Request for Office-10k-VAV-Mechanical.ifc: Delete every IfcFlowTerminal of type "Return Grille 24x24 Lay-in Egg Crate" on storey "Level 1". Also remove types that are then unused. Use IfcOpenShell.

First a look at what the model holds.

```python
import ifcopenshell
import ifcopenshell.util.element

model = ifcopenshell.open("Office-10k-VAV-Mechanical.ifc")
print(model.schema)
storey = next(s for s in model.by_type("IfcBuildingStorey") if s.Name == "Level 1")
terminals = [e for e in ifcopenshell.util.element.get_decomposition(storey) if e.is_a("IfcFlowTerminal")]
seen = {}
for e in terminals:
    element_type = ifcopenshell.util.element.get_type(e)
    name = element_type.Name if element_type not in (None, e) else None
    seen[name] = seen.get(name, 0) + 1
for name, count in sorted(seen.items(), key=str):
    print(count, "x", name)
```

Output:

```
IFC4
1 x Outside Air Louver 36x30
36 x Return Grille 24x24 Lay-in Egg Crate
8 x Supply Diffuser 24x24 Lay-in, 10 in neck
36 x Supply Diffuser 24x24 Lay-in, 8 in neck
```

```python
import ifcopenshell
import ifcopenshell.api.root
import ifcopenshell.util.element

model = ifcopenshell.open("Office-10k-VAV-Mechanical.ifc")

storey = next(s for s in model.by_type("IfcBuildingStorey") if s.Name == "Level 1")
terminals = [e for e in ifcopenshell.util.element.get_decomposition(storey) if e.is_a("IfcFlowTerminal")]
targets = [e for e in terminals if (t := ifcopenshell.util.element.get_type(e)) not in (None, e) and t.Name == "Return Grille 24x24 Lay-in Egg Crate"]
types = {ifcopenshell.util.element.get_type(e) for e in targets} - {None, *targets}

for e in targets:
    ifcopenshell.api.root.remove_product(model, product=e)
print(len(targets), "removed")

unused = [t for t in types if not ifcopenshell.util.element.get_types(t)]
for t in unused:
    ifcopenshell.api.root.remove_product(model, product=t)
print(len(unused), "unused types removed")

model.write("Office-10k-VAV-Mechanical_rev.ifc")
```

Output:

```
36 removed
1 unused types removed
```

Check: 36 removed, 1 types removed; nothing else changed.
